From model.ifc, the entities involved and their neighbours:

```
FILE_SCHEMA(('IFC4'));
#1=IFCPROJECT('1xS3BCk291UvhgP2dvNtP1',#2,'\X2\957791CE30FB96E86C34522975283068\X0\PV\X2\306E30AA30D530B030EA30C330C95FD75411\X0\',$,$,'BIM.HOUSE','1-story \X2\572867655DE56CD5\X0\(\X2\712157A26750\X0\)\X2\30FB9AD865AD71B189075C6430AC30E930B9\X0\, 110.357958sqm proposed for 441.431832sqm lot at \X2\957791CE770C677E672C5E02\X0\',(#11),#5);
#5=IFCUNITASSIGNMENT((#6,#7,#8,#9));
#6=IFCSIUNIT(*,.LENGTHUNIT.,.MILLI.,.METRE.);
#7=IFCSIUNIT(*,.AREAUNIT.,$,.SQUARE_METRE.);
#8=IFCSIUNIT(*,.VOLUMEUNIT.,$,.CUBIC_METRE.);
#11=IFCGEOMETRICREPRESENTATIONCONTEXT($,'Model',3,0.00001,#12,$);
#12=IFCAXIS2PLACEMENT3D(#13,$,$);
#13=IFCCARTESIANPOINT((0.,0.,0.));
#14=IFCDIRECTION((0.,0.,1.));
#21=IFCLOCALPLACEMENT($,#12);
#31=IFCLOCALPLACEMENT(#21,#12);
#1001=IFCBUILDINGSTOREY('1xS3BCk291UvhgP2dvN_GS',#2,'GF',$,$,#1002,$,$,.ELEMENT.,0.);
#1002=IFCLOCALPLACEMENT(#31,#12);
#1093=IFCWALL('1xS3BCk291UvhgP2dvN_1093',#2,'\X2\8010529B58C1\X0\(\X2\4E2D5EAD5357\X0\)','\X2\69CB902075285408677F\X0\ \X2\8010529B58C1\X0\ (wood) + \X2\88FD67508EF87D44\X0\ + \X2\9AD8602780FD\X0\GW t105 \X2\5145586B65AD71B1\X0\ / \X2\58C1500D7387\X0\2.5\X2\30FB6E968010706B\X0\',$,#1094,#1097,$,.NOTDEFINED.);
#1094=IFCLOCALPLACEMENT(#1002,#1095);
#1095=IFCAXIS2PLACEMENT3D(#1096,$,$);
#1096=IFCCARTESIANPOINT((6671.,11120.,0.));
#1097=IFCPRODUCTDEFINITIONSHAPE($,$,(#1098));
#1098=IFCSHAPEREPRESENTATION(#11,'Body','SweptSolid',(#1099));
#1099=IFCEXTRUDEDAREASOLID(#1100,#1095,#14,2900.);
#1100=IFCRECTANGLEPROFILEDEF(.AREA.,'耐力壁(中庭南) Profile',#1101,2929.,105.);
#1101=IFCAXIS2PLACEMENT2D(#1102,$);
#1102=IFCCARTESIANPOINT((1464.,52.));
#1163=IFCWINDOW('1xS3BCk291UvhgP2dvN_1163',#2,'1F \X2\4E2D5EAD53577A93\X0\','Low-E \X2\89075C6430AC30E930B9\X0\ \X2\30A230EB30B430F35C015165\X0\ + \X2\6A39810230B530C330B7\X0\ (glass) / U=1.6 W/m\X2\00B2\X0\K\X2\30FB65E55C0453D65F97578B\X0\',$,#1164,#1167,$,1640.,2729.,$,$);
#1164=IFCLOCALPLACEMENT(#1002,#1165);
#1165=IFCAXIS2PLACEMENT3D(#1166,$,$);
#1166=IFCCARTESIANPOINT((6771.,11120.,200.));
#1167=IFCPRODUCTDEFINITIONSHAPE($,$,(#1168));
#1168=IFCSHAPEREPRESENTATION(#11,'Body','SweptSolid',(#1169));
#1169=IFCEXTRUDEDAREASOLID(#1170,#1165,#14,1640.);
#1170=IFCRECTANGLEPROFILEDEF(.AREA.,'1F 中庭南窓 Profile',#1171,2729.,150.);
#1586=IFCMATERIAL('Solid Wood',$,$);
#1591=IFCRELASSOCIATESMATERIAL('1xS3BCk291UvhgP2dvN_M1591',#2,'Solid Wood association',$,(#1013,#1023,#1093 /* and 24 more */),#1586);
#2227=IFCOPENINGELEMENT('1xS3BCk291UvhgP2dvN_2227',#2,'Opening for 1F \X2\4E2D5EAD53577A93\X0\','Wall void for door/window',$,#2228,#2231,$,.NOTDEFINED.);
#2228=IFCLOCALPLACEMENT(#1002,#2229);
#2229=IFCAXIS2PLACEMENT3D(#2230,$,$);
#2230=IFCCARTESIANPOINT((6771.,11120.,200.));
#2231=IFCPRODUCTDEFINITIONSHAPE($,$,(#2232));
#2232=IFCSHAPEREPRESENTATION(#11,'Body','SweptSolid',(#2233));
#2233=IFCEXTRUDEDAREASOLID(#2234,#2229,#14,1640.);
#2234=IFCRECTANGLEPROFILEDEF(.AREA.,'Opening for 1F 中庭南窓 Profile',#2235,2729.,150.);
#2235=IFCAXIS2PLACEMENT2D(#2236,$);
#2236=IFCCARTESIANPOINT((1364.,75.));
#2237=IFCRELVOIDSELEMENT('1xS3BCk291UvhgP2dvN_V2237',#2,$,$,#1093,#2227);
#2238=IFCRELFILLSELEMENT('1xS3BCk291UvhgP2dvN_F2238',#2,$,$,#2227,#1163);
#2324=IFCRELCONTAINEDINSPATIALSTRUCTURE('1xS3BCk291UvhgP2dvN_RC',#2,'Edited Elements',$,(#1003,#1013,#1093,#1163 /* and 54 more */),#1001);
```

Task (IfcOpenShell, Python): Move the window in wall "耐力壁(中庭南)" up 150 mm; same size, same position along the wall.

```python
import numpy as np
import ifcopenshell
import ifcopenshell.api.geometry
import ifcopenshell.util.placement
import ifcopenshell.util.unit

model = ifcopenshell.open("model.ifc")
unit_scale = ifcopenshell.util.unit.calculate_unit_scale(model)

window = model.by_guid("1xS3BCk291UvhgP2dvN_1163")
opening = window.FillsVoids[0].RelatingOpeningElement
dz = 0.15 / unit_scale

shift = np.array([0.0, 0.0, dz])
# The window is not placed relative to its opening, so move both.
for product in (opening, window):
    matrix = ifcopenshell.util.placement.get_local_placement(product.ObjectPlacement)
    matrix[:3, 3] += shift
    ifcopenshell.api.geometry.edit_object_placement(model, product=product, matrix=matrix, is_si=False)

print(f"moved by {dz * unit_scale:+.3f} m")

model.write("model_rev.ifc")
```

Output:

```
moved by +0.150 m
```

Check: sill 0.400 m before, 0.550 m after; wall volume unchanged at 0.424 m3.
